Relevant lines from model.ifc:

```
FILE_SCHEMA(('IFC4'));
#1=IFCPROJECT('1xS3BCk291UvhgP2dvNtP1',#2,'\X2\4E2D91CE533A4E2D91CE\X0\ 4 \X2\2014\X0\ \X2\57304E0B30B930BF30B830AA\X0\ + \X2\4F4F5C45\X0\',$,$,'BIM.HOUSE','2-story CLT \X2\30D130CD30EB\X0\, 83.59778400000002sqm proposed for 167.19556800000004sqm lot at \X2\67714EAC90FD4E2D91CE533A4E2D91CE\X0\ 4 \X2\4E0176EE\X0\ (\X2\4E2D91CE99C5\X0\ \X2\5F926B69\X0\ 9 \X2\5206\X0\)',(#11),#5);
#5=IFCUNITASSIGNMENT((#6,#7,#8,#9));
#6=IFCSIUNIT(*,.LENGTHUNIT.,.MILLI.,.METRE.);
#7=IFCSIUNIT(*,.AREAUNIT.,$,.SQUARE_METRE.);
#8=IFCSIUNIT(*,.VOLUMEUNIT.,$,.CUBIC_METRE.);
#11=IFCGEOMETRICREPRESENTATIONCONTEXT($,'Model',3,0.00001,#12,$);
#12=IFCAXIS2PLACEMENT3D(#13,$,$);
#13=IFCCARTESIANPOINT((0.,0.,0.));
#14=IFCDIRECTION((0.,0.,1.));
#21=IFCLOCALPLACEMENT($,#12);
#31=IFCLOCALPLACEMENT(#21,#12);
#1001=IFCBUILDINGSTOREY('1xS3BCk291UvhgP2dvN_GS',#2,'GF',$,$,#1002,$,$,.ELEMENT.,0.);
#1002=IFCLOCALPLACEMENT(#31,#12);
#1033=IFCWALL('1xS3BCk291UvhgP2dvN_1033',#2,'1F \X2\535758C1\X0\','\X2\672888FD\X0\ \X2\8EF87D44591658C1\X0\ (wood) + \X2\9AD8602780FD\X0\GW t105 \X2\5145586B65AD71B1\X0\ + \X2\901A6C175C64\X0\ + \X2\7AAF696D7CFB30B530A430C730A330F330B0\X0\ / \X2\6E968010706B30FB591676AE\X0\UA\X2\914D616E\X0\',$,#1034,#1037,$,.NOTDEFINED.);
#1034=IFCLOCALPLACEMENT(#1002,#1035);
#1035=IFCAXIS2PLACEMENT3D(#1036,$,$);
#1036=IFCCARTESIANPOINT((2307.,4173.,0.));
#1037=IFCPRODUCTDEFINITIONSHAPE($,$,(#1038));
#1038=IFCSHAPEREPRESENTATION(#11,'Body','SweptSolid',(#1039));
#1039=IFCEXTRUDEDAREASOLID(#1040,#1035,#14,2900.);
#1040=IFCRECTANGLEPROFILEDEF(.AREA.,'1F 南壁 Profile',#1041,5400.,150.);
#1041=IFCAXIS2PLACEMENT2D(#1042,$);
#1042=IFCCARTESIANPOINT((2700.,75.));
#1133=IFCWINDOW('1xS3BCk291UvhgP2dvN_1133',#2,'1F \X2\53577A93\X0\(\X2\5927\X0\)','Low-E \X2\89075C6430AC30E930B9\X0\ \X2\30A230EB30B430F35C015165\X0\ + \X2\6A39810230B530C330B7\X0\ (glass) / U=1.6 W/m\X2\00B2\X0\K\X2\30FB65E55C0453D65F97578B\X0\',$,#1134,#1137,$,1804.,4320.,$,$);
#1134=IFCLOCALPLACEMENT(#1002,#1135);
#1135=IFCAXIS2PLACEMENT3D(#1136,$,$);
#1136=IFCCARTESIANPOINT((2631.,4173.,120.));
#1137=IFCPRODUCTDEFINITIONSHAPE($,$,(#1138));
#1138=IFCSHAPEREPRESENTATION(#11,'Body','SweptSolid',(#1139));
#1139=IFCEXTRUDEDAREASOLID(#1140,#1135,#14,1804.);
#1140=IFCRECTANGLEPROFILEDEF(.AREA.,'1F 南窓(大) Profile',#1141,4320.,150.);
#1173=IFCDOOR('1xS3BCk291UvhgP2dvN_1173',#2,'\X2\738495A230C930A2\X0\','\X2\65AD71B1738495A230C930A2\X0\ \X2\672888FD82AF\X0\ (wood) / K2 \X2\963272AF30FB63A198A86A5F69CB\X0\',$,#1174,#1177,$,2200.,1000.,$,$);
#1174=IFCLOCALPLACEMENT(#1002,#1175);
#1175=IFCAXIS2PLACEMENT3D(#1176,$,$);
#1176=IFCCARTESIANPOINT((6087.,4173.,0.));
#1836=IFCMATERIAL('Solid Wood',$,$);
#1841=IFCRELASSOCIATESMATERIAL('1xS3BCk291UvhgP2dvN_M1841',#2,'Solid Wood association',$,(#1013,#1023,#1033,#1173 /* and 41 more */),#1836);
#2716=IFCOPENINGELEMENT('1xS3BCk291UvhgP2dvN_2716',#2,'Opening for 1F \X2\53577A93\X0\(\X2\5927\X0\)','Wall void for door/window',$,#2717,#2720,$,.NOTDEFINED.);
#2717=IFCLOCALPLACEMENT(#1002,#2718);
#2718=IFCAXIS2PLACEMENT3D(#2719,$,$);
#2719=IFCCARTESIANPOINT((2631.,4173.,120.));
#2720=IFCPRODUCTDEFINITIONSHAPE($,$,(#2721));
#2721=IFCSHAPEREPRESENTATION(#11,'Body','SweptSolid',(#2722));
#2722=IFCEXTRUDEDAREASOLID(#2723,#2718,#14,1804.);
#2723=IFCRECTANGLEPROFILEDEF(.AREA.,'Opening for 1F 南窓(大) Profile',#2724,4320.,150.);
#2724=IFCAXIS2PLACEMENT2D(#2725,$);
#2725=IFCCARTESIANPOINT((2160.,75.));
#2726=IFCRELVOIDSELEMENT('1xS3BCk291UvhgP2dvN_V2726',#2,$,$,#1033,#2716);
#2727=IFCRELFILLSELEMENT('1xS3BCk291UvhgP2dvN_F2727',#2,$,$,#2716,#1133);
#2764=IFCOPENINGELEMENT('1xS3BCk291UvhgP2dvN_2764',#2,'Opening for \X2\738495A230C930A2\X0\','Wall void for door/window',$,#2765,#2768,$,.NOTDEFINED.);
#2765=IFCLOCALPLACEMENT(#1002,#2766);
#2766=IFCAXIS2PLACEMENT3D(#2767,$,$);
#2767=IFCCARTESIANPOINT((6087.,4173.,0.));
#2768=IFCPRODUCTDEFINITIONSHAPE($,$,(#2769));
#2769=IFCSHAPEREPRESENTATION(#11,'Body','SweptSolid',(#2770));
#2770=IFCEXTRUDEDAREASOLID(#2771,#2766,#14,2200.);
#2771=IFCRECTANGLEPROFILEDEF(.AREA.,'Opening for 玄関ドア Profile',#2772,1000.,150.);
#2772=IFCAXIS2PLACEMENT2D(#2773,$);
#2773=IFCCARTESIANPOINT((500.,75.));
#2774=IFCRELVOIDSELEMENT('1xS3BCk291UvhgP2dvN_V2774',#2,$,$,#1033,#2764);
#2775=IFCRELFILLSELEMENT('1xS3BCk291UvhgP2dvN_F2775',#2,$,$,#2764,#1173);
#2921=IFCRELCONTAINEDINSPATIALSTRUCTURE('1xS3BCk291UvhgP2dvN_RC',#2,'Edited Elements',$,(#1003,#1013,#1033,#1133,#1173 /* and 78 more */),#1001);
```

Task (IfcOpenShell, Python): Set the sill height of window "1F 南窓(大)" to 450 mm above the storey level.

```python
import numpy as np
import ifcopenshell
import ifcopenshell.api.geometry
import ifcopenshell.geom
import ifcopenshell.util.element
import ifcopenshell.util.placement
import ifcopenshell.util.shape
import ifcopenshell.util.unit

model = ifcopenshell.open("model.ifc")
unit_scale = ifcopenshell.util.unit.calculate_unit_scale(model)

window = model.by_guid("1xS3BCk291UvhgP2dvN_1133")
opening = window.FillsVoids[0].RelatingOpeningElement
storey = ifcopenshell.util.element.get_container(window, ifc_class="IfcBuildingStorey")
level = ifcopenshell.util.placement.get_local_placement(storey.ObjectPlacement)[2, 3]

# The opening's origin need not be at the sill, so measure its lowest point.
shape = ifcopenshell.geom.create_shape(ifcopenshell.geom.settings(), opening)
bottom = ifcopenshell.util.shape.get_shape_bottom_elevation(shape, shape.geometry) / unit_scale
dz = level + 450.0 - bottom

shift = np.array([0.0, 0.0, dz])
# The window is not placed relative to its opening, so move both.
for product in (opening, window):
    matrix = ifcopenshell.util.placement.get_local_placement(product.ObjectPlacement)
    matrix[:3, 3] += shift
    ifcopenshell.api.geometry.edit_object_placement(model, product=product, matrix=matrix, is_si=False)

print(f"moved by {dz * unit_scale:+.3f} m")

model.write("model_updated.ifc")
```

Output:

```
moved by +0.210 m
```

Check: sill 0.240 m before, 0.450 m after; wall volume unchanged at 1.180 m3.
